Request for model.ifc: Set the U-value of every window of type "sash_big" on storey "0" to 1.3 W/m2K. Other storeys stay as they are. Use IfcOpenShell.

First a look at what the model holds.

```python
import ifcopenshell
import ifcopenshell.util.element

model = ifcopenshell.open("model.ifc")
print(model.schema)
storey = next(s for s in model.by_type("IfcBuildingStorey") if s.Name == "0")
windows = [e for e in ifcopenshell.util.element.get_decomposition(storey) if e.is_a("IfcWindow")]
seen = {}
for e in windows:
    element_type = ifcopenshell.util.element.get_type(e)
    key = (element_type.Name if element_type != e and element_type else None, ifcopenshell.util.element.get_pset(e, "Pset_WindowCommon", "ThermalTransmittance"))
    seen[key] = seen.get(key, 0) + 1
for (name, value), count in sorted(seen.items(), key=str):
    print(count, "x", name, "|", value)
```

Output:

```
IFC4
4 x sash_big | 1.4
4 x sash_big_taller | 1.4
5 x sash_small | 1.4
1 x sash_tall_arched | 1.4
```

```python
import ifcopenshell
import ifcopenshell.api.pset
import ifcopenshell.util.element

model = ifcopenshell.open("model.ifc")

storey = next(s for s in model.by_type("IfcBuildingStorey") if s.Name == "0")
windows = [e for e in ifcopenshell.util.element.get_decomposition(storey) if e.is_a("IfcWindow")]

count = 0
for e in windows:
    element_type = ifcopenshell.util.element.get_type(e)
    if element_type in (None, e) or element_type.Name != "sash_big":
        continue
    # add_pset returns the element's existing set when there is one.
    pset = ifcopenshell.api.pset.add_pset(model, product=e, name="Pset_WindowCommon")
    ifcopenshell.api.pset.edit_pset(model, pset=pset, properties={"ThermalTransmittance": 1.3})
    count += 1

print(count, "windows updated")

model.write("model_updated.ifc")
```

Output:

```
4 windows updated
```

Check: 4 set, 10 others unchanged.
